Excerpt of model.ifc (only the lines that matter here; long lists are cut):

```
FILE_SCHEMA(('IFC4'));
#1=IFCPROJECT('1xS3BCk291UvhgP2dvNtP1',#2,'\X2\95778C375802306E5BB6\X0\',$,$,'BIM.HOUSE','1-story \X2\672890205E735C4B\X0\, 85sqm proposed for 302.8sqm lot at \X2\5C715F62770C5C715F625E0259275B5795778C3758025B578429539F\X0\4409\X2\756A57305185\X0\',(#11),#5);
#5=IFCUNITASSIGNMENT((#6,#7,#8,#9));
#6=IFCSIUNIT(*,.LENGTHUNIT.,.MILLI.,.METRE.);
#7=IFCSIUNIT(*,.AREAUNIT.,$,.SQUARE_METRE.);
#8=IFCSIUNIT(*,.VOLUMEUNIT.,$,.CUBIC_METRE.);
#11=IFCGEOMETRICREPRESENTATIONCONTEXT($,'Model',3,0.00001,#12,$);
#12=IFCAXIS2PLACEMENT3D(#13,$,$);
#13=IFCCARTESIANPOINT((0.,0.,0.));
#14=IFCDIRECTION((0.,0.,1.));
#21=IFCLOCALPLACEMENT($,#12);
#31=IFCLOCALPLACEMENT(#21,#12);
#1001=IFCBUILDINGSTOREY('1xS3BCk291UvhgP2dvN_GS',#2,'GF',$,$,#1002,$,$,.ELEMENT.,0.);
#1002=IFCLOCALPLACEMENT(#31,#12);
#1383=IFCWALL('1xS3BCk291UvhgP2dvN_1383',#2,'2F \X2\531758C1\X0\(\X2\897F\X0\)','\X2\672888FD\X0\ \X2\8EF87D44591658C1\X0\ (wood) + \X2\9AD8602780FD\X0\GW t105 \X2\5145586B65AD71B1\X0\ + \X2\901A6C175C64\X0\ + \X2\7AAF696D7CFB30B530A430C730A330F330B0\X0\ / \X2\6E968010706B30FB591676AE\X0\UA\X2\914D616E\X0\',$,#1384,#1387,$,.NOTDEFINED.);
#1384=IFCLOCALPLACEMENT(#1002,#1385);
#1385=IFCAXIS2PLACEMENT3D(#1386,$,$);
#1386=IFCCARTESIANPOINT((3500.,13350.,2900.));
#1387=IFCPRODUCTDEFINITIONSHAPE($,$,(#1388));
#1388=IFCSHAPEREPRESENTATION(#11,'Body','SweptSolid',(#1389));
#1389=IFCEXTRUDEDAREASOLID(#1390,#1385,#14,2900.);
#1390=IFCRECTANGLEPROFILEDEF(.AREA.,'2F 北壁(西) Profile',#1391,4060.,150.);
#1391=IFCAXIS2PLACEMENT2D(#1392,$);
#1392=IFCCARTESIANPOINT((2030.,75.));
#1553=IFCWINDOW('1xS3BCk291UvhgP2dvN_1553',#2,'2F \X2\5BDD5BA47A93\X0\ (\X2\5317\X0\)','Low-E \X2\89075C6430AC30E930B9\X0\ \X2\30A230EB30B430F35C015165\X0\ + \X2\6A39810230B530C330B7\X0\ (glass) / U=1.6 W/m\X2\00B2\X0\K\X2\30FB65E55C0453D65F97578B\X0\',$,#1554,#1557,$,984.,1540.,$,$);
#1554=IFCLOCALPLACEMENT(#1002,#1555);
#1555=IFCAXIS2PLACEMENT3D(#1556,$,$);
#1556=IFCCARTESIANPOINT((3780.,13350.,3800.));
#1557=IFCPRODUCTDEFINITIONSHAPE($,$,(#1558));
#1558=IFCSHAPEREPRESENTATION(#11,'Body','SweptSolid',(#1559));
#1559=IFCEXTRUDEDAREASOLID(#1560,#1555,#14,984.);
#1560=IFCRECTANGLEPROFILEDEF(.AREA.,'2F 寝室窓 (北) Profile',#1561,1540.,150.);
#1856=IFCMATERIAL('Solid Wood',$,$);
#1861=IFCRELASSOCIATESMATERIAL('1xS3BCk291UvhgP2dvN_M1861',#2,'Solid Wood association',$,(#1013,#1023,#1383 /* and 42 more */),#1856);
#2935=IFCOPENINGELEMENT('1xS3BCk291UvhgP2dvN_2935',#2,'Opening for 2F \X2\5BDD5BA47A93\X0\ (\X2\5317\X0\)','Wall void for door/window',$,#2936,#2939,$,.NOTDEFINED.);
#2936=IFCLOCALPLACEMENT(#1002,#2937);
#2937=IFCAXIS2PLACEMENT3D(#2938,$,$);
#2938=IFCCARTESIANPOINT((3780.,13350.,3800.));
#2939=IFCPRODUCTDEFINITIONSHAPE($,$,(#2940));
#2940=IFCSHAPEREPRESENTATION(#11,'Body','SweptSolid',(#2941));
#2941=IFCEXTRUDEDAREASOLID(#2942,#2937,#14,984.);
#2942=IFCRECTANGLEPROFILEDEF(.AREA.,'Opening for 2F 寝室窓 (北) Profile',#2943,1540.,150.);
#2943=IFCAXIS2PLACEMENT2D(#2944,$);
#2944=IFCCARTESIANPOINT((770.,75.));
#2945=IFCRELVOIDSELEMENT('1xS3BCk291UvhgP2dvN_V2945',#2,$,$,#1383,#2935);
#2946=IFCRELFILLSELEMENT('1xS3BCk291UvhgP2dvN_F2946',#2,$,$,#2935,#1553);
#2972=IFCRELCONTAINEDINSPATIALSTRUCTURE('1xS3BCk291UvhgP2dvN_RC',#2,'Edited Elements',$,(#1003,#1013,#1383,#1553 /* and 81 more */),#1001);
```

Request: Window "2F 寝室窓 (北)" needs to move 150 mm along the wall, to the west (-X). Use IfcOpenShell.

```python
import ifcopenshell
import ifcopenshell.api.geometry
import ifcopenshell.util.placement

model = ifcopenshell.open("model.ifc")

window = model.by_id(1553)
opening = window.FillsVoids[0].RelatingOpeningElement
wall = opening.VoidsElements[0].RelatingBuildingElement

wall_matrix = ifcopenshell.util.placement.get_local_placement(wall.ObjectPlacement)
shift = wall_matrix[:3, 0] * -150.0
before = ifcopenshell.util.placement.get_local_placement(window.ObjectPlacement)[:3, 3].copy()

# The window is not placed relative to its opening, so move both.
for product in (opening, window):
    matrix = ifcopenshell.util.placement.get_local_placement(product.ObjectPlacement)
    matrix[:3, 3] += shift
    ifcopenshell.api.geometry.edit_object_placement(model, product=product, matrix=matrix, is_si=False)

after = ifcopenshell.util.placement.get_local_placement(window.ObjectPlacement)[:3, 3]
print("window moved by", (after - before).round(3) + 0.0)

model.write("model_v2.ifc")
```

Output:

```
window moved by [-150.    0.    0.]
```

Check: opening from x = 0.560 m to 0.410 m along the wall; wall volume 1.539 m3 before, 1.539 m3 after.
